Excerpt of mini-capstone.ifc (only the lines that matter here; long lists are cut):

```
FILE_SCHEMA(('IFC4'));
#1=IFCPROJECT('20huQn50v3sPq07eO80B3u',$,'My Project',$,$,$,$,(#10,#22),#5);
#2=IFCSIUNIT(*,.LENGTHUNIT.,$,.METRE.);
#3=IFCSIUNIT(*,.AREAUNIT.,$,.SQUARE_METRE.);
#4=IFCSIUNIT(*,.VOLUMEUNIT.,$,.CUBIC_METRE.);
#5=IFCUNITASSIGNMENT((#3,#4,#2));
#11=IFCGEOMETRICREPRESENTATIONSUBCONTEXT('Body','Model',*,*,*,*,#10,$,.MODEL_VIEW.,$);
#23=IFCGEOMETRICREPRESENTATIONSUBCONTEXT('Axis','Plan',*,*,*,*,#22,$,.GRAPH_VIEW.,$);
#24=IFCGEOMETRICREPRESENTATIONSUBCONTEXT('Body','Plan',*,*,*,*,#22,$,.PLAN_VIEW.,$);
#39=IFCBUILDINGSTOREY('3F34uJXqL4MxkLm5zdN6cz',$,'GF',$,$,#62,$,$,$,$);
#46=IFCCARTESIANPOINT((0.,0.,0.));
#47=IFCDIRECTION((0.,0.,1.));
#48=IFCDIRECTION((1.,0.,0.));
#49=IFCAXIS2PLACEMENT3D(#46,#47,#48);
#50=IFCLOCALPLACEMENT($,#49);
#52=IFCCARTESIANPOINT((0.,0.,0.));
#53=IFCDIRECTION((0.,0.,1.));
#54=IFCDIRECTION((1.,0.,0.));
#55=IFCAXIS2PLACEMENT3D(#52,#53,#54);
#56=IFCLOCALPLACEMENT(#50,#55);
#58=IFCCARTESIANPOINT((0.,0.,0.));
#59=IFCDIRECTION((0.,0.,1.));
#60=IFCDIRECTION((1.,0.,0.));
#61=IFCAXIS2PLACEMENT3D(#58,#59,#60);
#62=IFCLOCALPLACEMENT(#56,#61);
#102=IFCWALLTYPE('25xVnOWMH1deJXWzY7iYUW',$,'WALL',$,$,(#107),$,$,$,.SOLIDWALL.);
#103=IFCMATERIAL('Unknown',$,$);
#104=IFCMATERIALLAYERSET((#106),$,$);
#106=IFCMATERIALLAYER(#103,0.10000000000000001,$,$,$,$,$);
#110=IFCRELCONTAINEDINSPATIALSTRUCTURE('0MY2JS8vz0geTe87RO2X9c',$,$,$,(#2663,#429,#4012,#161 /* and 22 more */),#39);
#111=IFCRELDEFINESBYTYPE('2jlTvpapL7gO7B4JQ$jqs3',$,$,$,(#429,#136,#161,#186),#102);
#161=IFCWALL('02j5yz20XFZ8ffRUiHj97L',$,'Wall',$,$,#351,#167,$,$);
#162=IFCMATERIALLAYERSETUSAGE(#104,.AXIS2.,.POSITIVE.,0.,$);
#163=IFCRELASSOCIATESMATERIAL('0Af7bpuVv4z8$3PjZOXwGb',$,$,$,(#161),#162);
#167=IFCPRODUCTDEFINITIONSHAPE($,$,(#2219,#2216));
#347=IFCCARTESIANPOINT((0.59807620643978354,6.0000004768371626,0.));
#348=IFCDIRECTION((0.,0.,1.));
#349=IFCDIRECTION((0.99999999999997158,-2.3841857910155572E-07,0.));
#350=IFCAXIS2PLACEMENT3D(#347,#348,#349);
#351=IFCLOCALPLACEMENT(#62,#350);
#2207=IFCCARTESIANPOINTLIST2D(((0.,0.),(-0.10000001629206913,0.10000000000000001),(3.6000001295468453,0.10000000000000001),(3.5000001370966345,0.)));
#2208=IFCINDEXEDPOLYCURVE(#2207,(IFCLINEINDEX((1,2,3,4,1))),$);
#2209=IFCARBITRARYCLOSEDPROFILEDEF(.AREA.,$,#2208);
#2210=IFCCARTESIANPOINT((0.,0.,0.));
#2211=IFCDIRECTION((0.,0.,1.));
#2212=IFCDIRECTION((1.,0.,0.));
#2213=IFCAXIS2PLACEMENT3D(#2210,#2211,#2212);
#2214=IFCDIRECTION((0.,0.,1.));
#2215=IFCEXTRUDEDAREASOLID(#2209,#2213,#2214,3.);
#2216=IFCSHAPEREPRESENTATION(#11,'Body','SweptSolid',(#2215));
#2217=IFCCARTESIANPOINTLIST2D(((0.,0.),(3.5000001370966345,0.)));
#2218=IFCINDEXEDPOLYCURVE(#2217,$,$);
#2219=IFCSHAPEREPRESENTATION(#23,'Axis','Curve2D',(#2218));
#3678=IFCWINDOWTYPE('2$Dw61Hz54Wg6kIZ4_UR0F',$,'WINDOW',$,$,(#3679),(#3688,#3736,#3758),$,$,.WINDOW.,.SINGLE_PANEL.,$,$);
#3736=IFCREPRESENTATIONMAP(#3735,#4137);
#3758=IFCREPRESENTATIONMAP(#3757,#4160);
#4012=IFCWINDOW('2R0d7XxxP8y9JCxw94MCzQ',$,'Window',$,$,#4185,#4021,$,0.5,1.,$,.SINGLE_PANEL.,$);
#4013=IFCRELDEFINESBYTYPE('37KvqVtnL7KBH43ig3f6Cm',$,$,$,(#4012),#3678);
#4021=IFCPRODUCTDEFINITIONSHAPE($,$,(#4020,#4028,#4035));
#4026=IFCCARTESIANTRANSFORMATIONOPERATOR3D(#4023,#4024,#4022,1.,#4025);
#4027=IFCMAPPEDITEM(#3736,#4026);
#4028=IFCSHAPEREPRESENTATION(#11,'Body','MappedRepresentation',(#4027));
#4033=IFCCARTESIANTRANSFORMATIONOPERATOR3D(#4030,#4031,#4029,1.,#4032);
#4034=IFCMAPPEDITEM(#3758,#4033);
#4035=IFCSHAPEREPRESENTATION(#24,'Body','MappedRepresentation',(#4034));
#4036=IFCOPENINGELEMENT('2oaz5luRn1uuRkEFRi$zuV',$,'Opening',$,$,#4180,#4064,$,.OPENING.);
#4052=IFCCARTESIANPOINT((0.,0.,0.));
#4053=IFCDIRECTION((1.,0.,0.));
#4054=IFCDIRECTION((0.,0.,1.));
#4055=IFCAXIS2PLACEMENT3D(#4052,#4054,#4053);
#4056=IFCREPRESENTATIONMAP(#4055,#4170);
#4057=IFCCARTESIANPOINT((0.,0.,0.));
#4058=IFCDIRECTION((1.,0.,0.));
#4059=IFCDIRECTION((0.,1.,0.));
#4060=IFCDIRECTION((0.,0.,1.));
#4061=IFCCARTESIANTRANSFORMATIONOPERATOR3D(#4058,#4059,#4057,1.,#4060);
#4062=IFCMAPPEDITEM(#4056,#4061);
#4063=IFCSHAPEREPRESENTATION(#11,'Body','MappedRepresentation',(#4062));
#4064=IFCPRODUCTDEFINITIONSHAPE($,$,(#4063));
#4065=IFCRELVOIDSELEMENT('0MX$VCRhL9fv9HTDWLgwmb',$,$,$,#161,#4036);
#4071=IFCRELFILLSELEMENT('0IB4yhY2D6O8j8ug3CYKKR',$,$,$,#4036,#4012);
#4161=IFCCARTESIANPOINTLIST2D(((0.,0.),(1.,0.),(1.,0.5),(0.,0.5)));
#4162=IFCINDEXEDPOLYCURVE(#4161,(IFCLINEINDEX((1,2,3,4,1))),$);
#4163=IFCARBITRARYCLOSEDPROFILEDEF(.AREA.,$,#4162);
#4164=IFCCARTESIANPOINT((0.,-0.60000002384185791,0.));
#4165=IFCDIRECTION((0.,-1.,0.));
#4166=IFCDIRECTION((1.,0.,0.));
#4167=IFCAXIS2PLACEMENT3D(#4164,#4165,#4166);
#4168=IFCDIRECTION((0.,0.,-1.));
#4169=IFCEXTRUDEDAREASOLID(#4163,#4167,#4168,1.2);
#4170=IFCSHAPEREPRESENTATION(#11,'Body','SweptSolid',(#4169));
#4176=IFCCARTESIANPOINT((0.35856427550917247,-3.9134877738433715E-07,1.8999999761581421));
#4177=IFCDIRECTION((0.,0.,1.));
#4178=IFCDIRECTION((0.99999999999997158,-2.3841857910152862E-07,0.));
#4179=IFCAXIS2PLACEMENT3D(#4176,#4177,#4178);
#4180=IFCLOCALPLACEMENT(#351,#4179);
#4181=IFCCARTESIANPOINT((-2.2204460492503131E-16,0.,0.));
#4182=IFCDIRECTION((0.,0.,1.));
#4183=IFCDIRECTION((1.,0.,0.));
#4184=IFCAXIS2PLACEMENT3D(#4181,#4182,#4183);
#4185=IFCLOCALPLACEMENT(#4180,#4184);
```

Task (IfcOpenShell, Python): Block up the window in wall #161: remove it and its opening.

```python
import ifcopenshell
import ifcopenshell.api.feature
import ifcopenshell.api.root
import ifcopenshell.geom
import ifcopenshell.util.shape

model = ifcopenshell.open("mini-capstone.ifc")
settings = ifcopenshell.geom.settings()


def volume(element):
    """Net volume in cubic metres, openings subtracted."""
    shape = ifcopenshell.geom.create_shape(settings, element)
    return ifcopenshell.util.shape.get_volume(shape.geometry)


window = model.by_guid("2R0d7XxxP8y9JCxw94MCzQ")
opening = window.FillsVoids[0].RelatingOpeningElement
wall = opening.VoidsElements[0].RelatingBuildingElement
before = volume(wall)

ifcopenshell.api.root.remove_product(model, product=window)
ifcopenshell.api.feature.remove_feature(model, feature=opening)

after = volume(wall)

print(f"wall volume {before:.3f} -> {after:.3f} m3")

model.write("mini-capstone_v2.ifc")
```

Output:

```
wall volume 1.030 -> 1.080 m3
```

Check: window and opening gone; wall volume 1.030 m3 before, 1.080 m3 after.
